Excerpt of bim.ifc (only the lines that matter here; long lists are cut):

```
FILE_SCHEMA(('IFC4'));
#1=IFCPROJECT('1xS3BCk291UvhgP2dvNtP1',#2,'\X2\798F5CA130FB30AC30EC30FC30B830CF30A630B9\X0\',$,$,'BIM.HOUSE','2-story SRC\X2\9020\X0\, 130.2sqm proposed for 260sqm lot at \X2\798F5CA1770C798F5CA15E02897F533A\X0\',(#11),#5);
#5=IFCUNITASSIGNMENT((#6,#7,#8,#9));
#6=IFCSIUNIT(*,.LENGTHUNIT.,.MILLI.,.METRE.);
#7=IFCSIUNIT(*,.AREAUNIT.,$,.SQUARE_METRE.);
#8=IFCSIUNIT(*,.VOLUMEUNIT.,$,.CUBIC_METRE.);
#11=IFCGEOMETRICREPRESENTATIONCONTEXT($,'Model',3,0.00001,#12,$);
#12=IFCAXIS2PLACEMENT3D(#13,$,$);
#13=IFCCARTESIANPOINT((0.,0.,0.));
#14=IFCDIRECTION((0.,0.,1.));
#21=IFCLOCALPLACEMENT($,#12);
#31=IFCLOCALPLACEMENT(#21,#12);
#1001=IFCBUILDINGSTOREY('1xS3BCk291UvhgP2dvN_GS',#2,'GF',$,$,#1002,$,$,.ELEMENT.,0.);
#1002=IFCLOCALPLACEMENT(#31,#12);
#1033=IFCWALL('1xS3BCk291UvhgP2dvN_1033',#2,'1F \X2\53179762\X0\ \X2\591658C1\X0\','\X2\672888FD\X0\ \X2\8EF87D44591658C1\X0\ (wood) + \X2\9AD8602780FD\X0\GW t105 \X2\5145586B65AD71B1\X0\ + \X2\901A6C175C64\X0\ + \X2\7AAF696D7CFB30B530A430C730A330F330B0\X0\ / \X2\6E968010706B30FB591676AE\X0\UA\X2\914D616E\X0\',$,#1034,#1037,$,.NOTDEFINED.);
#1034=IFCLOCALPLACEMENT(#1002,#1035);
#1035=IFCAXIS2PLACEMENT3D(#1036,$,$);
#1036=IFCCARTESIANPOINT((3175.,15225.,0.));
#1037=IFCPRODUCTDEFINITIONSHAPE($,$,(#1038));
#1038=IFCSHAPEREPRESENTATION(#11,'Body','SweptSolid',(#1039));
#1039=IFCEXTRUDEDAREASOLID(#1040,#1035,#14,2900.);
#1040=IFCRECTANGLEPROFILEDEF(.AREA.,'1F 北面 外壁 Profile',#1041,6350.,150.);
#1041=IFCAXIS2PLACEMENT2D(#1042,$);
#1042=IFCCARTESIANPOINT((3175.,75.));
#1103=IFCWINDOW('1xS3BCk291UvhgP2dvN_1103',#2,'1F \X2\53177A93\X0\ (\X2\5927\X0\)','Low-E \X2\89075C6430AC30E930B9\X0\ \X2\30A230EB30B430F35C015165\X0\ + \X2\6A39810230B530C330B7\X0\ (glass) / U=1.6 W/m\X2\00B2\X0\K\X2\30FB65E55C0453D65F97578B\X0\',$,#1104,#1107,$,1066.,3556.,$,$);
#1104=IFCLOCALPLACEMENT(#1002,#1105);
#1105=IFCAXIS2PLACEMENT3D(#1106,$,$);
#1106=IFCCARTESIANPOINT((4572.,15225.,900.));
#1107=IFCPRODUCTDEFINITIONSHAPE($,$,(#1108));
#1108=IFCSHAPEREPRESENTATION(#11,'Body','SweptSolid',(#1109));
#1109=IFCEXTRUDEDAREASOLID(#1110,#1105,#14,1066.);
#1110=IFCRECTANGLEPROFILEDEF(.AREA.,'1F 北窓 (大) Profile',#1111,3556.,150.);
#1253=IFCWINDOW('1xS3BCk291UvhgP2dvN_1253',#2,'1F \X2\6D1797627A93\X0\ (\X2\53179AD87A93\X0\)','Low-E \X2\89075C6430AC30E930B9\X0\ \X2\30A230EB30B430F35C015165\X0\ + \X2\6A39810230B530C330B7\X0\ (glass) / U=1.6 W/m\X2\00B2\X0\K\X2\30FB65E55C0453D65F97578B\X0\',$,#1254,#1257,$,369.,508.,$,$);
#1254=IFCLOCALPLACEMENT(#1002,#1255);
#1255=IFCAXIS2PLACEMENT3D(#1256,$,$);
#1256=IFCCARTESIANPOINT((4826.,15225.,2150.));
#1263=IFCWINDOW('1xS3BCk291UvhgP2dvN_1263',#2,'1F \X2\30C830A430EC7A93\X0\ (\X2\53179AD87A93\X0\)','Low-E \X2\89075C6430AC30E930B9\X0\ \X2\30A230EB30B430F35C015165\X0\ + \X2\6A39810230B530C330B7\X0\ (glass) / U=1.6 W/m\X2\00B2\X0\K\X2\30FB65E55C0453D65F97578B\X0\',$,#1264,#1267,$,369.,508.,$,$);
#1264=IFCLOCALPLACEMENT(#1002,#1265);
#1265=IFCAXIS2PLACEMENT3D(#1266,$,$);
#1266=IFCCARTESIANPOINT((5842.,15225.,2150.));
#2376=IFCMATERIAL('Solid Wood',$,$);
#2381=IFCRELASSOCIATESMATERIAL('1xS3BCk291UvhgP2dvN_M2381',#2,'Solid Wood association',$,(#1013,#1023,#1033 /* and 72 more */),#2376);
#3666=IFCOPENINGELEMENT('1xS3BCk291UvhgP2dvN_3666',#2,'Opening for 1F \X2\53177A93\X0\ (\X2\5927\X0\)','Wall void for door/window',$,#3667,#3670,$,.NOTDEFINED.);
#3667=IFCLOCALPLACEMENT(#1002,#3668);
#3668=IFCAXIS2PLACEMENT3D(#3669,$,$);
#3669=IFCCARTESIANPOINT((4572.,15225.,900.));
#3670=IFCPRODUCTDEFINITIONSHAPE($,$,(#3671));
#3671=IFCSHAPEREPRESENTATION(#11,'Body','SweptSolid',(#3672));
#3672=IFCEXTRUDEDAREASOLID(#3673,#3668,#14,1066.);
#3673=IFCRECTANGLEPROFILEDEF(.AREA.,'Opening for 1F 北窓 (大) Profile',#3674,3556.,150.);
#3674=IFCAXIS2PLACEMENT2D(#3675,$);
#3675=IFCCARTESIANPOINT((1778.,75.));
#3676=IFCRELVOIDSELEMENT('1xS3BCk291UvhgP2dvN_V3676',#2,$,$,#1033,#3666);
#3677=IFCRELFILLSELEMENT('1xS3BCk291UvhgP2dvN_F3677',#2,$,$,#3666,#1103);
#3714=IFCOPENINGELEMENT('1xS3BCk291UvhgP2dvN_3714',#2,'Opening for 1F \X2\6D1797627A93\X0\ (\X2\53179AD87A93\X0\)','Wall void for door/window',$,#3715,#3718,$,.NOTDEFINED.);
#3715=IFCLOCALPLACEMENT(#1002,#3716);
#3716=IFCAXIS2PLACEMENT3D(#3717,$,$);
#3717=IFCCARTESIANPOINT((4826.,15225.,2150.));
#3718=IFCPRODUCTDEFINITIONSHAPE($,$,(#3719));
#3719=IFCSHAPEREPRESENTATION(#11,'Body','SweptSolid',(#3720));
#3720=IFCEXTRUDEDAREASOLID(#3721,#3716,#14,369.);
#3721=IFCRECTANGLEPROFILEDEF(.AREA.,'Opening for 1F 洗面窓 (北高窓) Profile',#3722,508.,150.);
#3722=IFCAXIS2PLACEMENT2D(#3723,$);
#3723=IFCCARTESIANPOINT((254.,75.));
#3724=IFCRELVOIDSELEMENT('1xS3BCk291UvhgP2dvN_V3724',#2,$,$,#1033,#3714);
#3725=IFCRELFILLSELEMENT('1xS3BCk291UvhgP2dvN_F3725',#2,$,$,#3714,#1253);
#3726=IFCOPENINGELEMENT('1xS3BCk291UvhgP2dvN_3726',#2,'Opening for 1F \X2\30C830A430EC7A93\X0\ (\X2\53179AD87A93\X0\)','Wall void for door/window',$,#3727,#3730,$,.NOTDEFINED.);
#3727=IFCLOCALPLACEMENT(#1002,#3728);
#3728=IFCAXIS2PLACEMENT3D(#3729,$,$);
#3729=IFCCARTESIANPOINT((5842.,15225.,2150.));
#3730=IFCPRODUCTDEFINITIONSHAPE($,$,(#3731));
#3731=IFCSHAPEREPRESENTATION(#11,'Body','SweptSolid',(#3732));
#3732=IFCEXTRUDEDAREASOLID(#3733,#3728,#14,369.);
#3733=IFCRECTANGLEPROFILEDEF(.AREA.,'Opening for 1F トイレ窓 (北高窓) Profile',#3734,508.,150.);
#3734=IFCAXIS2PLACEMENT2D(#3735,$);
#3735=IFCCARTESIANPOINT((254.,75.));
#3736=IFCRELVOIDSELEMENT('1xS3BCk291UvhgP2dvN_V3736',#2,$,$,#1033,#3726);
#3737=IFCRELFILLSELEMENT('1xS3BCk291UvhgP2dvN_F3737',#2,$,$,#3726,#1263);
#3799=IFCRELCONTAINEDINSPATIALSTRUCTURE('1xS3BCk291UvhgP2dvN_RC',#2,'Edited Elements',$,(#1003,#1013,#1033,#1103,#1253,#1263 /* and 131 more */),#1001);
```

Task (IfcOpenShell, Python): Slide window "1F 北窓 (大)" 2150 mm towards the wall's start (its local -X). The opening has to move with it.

```python
import ifcopenshell
import ifcopenshell.api.geometry
import ifcopenshell.util.placement

model = ifcopenshell.open("bim.ifc")

window = model.by_guid("1xS3BCk291UvhgP2dvN_1103")
opening = window.FillsVoids[0].RelatingOpeningElement
wall = opening.VoidsElements[0].RelatingBuildingElement

wall_matrix = ifcopenshell.util.placement.get_local_placement(wall.ObjectPlacement)
shift = wall_matrix[:3, 0] * -2150.0
before = ifcopenshell.util.placement.get_local_placement(window.ObjectPlacement)[:3, 3].copy()

# The window is not placed relative to its opening, so move both.
for product in (opening, window):
    matrix = ifcopenshell.util.placement.get_local_placement(product.ObjectPlacement)
    matrix[:3, 3] += shift
    ifcopenshell.api.geometry.edit_object_placement(model, product=product, matrix=matrix, is_si=False)

after = ifcopenshell.util.placement.get_local_placement(window.ObjectPlacement)[:3, 3]
print("window moved by", (after - before).round(3) + 0.0)

model.write("bim-out.ifc")
```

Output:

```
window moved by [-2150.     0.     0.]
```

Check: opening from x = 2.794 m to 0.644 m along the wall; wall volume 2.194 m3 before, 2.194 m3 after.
